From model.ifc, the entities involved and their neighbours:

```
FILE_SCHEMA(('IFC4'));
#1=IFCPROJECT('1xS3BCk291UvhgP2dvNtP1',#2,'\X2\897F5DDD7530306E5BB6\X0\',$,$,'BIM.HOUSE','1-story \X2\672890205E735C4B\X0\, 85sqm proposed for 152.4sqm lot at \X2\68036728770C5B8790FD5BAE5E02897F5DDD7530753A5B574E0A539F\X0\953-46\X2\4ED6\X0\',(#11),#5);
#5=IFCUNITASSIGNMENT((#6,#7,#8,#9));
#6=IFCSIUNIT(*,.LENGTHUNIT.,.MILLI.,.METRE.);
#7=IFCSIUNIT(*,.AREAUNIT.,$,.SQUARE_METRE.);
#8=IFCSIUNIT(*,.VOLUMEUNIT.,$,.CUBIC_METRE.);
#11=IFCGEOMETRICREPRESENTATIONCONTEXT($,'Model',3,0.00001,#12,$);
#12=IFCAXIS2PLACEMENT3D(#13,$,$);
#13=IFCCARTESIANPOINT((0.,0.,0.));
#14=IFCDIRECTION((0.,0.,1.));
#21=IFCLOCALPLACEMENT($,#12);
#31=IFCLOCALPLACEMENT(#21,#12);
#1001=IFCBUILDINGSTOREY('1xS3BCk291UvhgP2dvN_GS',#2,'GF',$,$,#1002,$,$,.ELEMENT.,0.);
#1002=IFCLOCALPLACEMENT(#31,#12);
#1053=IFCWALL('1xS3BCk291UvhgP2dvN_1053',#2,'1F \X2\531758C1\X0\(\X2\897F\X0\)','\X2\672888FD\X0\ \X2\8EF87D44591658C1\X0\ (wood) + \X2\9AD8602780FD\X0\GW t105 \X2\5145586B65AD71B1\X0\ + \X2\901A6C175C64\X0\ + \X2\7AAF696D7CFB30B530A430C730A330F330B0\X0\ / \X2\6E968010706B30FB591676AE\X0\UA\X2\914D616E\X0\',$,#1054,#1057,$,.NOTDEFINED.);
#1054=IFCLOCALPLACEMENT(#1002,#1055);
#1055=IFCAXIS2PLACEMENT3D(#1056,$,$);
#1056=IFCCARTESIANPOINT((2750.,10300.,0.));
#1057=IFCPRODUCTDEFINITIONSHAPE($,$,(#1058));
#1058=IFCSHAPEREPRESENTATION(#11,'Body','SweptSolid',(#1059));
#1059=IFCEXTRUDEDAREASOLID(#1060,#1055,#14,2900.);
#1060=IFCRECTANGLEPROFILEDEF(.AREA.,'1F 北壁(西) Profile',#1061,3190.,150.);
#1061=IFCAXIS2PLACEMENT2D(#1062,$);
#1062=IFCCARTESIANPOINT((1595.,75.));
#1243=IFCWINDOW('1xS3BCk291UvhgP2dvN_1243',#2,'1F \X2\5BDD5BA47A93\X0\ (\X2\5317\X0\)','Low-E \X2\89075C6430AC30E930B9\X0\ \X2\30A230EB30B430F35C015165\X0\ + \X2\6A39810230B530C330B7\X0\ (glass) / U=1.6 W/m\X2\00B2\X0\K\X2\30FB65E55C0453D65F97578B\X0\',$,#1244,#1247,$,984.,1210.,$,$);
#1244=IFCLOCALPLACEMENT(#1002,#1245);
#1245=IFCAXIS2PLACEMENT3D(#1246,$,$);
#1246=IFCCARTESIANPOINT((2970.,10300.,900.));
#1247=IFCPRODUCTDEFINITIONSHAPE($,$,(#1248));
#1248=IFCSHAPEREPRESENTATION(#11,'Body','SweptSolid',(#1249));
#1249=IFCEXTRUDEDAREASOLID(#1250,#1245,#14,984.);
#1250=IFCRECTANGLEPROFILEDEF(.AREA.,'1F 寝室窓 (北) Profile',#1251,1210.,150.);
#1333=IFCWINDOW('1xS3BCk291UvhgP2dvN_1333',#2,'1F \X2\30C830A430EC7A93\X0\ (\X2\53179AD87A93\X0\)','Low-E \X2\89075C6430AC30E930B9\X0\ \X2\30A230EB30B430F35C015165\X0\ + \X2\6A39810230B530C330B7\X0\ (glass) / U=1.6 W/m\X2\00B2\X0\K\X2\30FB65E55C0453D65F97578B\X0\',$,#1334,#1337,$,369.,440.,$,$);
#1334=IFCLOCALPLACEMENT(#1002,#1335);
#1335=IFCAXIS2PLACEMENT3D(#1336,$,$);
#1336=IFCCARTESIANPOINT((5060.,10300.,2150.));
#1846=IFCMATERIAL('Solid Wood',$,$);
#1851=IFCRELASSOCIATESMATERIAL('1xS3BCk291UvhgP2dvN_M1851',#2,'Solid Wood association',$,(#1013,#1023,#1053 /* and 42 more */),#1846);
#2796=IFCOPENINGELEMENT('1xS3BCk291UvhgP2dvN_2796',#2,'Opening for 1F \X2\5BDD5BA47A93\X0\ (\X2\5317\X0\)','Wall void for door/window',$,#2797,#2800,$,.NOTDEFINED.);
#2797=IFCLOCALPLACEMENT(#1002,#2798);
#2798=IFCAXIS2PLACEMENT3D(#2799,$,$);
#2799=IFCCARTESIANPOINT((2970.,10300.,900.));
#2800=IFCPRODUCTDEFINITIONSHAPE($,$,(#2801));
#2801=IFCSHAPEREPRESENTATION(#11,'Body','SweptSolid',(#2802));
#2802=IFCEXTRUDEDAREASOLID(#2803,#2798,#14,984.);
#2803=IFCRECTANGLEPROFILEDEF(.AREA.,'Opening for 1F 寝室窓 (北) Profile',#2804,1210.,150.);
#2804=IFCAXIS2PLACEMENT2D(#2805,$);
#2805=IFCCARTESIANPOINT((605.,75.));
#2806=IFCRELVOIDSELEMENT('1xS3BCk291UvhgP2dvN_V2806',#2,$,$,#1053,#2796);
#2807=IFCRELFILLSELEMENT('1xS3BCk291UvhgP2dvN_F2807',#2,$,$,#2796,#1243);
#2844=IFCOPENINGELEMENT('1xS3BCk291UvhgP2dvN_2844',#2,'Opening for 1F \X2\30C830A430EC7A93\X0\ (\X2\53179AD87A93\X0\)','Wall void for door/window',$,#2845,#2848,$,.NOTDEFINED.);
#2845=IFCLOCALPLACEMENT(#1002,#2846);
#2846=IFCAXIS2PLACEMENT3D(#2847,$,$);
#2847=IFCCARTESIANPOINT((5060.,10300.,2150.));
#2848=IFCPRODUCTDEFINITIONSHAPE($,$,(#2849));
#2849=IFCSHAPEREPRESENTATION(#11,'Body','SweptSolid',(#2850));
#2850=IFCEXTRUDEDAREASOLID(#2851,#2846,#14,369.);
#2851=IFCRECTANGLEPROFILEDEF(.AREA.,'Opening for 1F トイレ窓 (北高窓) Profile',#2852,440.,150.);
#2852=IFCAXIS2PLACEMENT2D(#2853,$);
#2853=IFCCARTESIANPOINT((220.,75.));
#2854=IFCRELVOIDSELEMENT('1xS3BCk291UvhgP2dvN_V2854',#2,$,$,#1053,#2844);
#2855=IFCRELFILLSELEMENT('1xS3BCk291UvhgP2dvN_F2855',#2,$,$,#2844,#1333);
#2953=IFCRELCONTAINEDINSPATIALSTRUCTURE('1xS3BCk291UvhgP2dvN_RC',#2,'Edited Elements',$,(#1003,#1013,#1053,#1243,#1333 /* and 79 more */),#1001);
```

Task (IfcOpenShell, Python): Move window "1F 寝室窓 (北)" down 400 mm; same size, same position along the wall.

```python
import numpy as np
import ifcopenshell
import ifcopenshell.api.geometry
import ifcopenshell.util.placement
import ifcopenshell.util.unit

model = ifcopenshell.open("model.ifc")
unit_scale = ifcopenshell.util.unit.calculate_unit_scale(model)

window = model.by_guid("1xS3BCk291UvhgP2dvN_1243")
opening = window.FillsVoids[0].RelatingOpeningElement
dz = -0.4 / unit_scale

shift = np.array([0.0, 0.0, dz])
# The window is not placed relative to its opening, so move both.
for product in (opening, window):
    matrix = ifcopenshell.util.placement.get_local_placement(product.ObjectPlacement)
    matrix[:3, 3] += shift
    ifcopenshell.api.geometry.edit_object_placement(model, product=product, matrix=matrix, is_si=False)

print(f"moved by {dz * unit_scale:+.3f} m")

model.write("model_edited.ifc")
```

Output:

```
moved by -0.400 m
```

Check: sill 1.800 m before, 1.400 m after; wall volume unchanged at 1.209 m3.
